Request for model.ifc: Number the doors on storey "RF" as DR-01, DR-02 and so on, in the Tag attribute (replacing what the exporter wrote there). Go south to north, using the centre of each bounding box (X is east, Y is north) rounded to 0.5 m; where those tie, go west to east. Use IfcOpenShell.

First a look at what the model holds.

```python
import ifcopenshell
import ifcopenshell.util.element
import ifcopenshell.util.placement

model = ifcopenshell.open("model.ifc")
print(model.schema)
storey = next(s for s in model.by_type("IfcBuildingStorey") if s.Name == "RF")
doors = [e for e in ifcopenshell.util.element.get_decomposition(storey) if e.is_a("IfcDoor")]
for e in sorted(doors, key=lambda e: e.id()):
    origin = ifcopenshell.util.placement.get_local_placement(e.ObjectPlacement)[:3, 3]
    print(e.id(), e.Tag, e.Name, origin.round(2) + 0.0, sep=" | ")
```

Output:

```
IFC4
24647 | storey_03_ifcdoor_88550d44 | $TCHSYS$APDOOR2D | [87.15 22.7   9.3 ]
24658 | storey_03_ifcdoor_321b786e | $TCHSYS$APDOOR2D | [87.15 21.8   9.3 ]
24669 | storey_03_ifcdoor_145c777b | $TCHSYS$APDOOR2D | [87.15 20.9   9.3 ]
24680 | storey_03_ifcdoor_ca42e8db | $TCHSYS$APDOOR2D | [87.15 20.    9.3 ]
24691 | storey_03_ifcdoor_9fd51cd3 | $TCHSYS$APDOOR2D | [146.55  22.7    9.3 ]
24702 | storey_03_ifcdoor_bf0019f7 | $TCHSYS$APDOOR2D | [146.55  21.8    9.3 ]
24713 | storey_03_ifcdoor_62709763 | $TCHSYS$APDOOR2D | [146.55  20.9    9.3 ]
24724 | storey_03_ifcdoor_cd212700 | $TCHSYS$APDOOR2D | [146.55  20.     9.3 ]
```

```python
import ifcopenshell
import ifcopenshell.geom
import ifcopenshell.util.element
import ifcopenshell.util.shape

model = ifcopenshell.open("model.ifc")
settings = ifcopenshell.geom.settings()
settings.set("use-world-coords", True)


def centre(element):
    shape = ifcopenshell.geom.create_shape(settings, element)
    return ifcopenshell.util.shape.get_bbox_centroid(shape.geometry)


storey = next(s for s in model.by_type("IfcBuildingStorey") if s.Name == "RF")
doors = [e for e in ifcopenshell.util.element.get_decomposition(storey) if e.is_a("IfcDoor")]

# Insertion points can sit at a corner or the storey origin, so sort by the geometry (in metres).
centres = {e: centre(e) for e in doors}
doors.sort(key=lambda e: (round(centres[e][1] / 0.5), centres[e][0]))

for i, e in enumerate(doors, start=1):
    number = f"DR-{i:02d}"
    e.Tag = number
    print(e.id(), number)

model.write("model_rev.ifc")
```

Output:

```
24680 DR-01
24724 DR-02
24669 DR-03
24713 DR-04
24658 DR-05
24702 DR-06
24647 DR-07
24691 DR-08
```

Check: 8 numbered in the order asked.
